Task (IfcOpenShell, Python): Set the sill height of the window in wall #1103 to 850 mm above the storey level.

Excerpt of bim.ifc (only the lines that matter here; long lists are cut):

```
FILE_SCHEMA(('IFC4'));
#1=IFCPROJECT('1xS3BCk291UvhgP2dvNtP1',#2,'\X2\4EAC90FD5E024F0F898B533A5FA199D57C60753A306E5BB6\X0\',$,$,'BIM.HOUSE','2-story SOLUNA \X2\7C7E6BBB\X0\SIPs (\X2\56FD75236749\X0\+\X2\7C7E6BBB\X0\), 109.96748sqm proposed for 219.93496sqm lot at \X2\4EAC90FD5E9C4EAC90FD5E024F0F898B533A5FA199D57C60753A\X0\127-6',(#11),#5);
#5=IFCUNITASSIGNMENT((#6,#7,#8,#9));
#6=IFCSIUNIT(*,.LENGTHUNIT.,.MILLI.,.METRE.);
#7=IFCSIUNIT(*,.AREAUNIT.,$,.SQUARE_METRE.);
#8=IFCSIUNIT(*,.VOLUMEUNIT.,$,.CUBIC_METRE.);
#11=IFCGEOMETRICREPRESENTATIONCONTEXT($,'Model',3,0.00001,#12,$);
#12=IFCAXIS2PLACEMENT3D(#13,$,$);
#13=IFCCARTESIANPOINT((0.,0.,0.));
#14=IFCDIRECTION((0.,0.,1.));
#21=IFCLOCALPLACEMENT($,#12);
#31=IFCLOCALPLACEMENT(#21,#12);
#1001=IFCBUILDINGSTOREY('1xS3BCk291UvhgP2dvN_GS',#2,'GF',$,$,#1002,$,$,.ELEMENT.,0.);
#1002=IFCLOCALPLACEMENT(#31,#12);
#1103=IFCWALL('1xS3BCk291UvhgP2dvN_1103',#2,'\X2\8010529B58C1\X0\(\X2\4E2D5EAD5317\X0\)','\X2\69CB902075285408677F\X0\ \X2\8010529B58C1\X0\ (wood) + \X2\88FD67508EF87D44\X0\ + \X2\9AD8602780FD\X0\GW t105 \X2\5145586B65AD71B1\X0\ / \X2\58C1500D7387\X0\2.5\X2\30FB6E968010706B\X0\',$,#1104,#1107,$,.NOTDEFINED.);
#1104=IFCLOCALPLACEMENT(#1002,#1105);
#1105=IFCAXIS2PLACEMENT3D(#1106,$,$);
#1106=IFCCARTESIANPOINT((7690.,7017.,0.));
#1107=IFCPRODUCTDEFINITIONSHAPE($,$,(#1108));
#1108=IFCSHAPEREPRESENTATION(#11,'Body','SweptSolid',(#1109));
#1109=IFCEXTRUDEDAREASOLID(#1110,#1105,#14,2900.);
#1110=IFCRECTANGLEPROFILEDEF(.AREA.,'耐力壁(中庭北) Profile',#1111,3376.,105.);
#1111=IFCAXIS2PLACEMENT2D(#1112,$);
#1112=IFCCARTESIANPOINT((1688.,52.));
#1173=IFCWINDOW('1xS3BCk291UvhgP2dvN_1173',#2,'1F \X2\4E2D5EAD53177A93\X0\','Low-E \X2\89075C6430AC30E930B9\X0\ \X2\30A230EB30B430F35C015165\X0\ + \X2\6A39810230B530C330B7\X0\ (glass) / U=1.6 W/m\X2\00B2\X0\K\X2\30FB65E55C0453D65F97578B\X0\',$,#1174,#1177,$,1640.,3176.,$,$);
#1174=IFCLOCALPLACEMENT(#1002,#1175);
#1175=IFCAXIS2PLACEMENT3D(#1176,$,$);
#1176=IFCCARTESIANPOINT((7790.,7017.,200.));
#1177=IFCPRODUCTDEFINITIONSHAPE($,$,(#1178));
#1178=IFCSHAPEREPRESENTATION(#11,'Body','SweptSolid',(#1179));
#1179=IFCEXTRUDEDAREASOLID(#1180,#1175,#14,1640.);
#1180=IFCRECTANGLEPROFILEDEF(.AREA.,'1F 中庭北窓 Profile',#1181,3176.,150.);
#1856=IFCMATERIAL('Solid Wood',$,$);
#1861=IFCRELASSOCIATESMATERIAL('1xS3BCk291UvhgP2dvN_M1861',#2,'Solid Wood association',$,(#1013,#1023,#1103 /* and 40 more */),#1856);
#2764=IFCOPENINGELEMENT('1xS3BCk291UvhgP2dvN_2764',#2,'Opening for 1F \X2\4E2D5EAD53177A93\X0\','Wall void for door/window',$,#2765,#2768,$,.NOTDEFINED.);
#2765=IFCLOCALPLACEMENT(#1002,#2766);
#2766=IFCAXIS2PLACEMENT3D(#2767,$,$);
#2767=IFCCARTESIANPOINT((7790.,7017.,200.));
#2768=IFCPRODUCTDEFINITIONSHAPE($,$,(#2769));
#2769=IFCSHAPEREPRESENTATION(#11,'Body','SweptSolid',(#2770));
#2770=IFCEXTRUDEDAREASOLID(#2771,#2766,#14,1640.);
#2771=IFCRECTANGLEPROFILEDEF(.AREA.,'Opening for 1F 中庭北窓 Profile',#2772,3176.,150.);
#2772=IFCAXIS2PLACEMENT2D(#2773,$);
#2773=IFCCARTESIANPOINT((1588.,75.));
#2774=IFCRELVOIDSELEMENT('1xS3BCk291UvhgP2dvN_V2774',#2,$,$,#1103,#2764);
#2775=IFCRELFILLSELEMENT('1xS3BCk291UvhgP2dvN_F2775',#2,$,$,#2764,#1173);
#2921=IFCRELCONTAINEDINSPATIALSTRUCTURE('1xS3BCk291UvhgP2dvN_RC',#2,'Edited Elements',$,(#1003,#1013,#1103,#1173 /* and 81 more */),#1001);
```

```python
import numpy as np
import ifcopenshell
import ifcopenshell.api.geometry
import ifcopenshell.geom
import ifcopenshell.util.element
import ifcopenshell.util.placement
import ifcopenshell.util.shape
import ifcopenshell.util.unit

model = ifcopenshell.open("bim.ifc")
unit_scale = ifcopenshell.util.unit.calculate_unit_scale(model)

window = model.by_id(1173)
opening = window.FillsVoids[0].RelatingOpeningElement
storey = ifcopenshell.util.element.get_container(window, ifc_class="IfcBuildingStorey")
level = ifcopenshell.util.placement.get_local_placement(storey.ObjectPlacement)[2, 3]

# The opening's origin need not be at the sill, so measure its lowest point.
shape = ifcopenshell.geom.create_shape(ifcopenshell.geom.settings(), opening)
bottom = ifcopenshell.util.shape.get_shape_bottom_elevation(shape, shape.geometry) / unit_scale
dz = level + 850.0 - bottom

shift = np.array([0.0, 0.0, dz])
# The window is not placed relative to its opening, so move both.
for product in (opening, window):
    matrix = ifcopenshell.util.placement.get_local_placement(product.ObjectPlacement)
    matrix[:3, 3] += shift
    ifcopenshell.api.geometry.edit_object_placement(model, product=product, matrix=matrix, is_si=False)

print(f"moved by {dz * unit_scale:+.3f} m")

model.write("bim_rev.ifc")
```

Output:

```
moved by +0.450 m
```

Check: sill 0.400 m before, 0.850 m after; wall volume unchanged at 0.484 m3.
